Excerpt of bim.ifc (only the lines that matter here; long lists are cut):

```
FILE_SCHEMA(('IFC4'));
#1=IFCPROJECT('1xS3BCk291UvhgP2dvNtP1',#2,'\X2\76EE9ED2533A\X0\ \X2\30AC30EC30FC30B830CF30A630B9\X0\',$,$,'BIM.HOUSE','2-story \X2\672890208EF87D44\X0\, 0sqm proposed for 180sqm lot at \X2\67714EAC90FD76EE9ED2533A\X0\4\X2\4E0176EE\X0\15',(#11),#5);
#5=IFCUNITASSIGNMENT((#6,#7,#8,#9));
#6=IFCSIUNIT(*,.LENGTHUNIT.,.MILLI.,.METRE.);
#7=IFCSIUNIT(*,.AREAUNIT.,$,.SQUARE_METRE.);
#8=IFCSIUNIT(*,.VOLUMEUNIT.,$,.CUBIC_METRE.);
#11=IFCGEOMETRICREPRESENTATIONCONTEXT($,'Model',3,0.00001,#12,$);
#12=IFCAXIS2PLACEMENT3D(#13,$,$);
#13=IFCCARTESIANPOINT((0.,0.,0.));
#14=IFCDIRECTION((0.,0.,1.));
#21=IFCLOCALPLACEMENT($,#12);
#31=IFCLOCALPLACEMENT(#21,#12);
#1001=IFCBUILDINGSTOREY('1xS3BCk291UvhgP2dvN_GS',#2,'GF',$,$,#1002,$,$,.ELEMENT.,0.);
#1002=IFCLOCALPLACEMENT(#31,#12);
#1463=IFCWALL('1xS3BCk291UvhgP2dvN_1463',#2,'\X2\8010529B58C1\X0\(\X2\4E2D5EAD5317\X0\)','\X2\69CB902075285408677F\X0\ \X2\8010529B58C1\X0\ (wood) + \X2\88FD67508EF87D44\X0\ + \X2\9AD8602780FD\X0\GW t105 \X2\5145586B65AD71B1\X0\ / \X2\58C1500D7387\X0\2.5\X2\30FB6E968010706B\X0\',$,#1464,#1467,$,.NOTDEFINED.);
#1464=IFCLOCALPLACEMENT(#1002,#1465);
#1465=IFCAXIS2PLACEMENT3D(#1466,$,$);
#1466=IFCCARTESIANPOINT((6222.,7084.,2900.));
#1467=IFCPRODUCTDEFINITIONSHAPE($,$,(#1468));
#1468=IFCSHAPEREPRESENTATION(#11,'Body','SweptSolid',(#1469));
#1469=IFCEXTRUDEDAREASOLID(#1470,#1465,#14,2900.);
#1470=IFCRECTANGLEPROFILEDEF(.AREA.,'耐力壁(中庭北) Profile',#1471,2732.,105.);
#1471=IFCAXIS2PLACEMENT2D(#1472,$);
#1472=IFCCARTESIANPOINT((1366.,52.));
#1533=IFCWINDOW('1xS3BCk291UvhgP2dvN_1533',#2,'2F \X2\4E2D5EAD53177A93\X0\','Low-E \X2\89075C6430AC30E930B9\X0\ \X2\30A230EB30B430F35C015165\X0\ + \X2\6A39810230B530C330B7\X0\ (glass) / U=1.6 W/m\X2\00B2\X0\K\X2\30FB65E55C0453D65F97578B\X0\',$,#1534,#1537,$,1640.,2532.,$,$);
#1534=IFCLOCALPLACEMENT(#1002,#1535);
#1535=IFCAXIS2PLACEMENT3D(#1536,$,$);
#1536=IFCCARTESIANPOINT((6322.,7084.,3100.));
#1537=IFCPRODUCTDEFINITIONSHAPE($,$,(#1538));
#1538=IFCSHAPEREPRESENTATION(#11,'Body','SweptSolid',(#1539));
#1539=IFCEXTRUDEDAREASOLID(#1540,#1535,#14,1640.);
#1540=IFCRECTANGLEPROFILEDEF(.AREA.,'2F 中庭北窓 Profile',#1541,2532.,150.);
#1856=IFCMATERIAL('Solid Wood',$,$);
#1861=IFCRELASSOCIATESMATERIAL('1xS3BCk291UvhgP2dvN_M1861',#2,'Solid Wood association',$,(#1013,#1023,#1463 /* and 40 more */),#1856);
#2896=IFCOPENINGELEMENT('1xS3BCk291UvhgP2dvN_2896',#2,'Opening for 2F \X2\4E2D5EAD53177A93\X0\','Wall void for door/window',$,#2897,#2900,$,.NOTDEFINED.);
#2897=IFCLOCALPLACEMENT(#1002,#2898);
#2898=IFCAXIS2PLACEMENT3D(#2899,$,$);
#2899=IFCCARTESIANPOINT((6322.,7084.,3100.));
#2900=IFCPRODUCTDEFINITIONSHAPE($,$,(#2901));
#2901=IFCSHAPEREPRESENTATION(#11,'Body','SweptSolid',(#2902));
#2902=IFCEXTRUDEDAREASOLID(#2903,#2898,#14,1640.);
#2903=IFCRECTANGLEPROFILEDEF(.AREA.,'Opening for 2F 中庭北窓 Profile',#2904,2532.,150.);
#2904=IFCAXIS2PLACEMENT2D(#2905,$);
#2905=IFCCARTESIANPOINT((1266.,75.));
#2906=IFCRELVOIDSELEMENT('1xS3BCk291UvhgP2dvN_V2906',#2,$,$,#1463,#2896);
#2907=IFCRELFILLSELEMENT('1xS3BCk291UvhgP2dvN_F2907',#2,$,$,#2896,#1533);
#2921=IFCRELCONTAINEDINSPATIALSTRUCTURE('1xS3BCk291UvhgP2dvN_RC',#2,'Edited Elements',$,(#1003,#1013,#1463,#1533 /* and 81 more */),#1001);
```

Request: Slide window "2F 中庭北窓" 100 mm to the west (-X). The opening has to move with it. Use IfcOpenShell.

```python
import ifcopenshell
import ifcopenshell.api.geometry
import ifcopenshell.util.placement

model = ifcopenshell.open("bim.ifc")

window = model.by_guid("1xS3BCk291UvhgP2dvN_1533")
opening = window.FillsVoids[0].RelatingOpeningElement
wall = opening.VoidsElements[0].RelatingBuildingElement

wall_matrix = ifcopenshell.util.placement.get_local_placement(wall.ObjectPlacement)
shift = wall_matrix[:3, 0] * -100.0
before = ifcopenshell.util.placement.get_local_placement(window.ObjectPlacement)[:3, 3].copy()

# The window is not placed relative to its opening, so move both.
for product in (opening, window):
    matrix = ifcopenshell.util.placement.get_local_placement(product.ObjectPlacement)
    matrix[:3, 3] += shift
    ifcopenshell.api.geometry.edit_object_placement(model, product=product, matrix=matrix, is_si=False)

after = ifcopenshell.util.placement.get_local_placement(window.ObjectPlacement)[:3, 3]
print("window moved by", (after - before).round(3) + 0.0)

model.write("bim_rev.ifc")
```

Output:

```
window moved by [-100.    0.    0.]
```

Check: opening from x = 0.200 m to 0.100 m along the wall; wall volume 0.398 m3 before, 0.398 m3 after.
